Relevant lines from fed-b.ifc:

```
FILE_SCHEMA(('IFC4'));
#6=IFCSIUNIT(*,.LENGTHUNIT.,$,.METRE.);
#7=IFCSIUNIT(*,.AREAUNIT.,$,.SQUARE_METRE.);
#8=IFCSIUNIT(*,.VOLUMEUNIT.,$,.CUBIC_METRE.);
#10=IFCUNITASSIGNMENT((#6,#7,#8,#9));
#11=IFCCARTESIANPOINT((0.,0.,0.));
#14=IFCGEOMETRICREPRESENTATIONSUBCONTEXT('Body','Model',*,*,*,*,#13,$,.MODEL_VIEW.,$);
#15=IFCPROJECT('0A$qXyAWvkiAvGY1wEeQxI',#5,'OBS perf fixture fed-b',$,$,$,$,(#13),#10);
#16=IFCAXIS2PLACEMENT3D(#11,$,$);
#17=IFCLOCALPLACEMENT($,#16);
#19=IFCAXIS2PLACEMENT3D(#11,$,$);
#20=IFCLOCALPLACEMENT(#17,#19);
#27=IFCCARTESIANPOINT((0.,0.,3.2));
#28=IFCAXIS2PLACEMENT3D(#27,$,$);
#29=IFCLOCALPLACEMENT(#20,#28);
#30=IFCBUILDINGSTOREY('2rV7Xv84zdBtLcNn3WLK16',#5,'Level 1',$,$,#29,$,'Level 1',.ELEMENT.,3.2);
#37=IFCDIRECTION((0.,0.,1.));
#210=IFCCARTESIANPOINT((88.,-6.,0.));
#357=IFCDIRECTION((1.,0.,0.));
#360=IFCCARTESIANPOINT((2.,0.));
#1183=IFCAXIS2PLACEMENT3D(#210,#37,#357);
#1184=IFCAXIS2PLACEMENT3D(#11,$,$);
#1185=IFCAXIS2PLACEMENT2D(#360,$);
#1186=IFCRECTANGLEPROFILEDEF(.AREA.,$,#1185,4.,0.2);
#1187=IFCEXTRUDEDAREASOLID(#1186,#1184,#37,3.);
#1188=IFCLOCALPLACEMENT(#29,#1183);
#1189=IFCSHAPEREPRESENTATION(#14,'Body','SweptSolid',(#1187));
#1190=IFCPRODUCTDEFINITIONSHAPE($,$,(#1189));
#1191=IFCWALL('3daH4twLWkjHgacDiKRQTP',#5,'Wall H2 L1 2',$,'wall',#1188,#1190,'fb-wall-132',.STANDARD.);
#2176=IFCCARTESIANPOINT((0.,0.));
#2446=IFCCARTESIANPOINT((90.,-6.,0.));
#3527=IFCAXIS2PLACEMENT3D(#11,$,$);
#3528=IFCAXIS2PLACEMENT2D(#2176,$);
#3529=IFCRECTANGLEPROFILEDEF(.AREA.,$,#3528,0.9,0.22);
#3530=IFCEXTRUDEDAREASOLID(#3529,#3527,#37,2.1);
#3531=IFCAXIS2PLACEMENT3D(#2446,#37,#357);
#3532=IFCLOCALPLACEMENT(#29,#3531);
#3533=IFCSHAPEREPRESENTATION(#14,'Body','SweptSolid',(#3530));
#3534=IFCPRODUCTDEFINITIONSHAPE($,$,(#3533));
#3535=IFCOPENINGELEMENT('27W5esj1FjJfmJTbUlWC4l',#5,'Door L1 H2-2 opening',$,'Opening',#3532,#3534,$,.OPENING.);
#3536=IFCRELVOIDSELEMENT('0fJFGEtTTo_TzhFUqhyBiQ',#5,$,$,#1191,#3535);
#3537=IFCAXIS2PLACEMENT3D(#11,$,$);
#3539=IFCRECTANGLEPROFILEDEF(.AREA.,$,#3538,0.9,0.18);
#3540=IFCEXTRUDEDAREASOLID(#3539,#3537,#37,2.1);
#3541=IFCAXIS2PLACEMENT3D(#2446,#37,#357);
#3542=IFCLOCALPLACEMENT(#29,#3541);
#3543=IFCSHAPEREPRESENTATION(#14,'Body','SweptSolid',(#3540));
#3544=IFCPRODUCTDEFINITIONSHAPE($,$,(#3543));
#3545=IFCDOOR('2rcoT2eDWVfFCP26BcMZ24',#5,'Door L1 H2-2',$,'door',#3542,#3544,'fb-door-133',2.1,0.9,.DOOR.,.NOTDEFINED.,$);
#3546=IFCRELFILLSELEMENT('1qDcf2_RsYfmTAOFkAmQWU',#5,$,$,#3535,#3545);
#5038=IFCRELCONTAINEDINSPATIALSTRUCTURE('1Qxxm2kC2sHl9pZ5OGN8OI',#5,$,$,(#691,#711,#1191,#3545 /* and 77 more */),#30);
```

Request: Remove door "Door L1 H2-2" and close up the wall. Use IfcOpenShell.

```python
import ifcopenshell
import ifcopenshell.api.feature
import ifcopenshell.api.root
import ifcopenshell.geom
import ifcopenshell.util.shape

model = ifcopenshell.open("fed-b.ifc")
settings = ifcopenshell.geom.settings()


def volume(element):
    """Net volume in cubic metres, openings subtracted."""
    shape = ifcopenshell.geom.create_shape(settings, element)
    return ifcopenshell.util.shape.get_volume(shape.geometry)


door = model.by_guid("2rcoT2eDWVfFCP26BcMZ24")
opening = door.FillsVoids[0].RelatingOpeningElement
wall = opening.VoidsElements[0].RelatingBuildingElement
before = volume(wall)

ifcopenshell.api.root.remove_product(model, product=door)
ifcopenshell.api.feature.remove_feature(model, feature=opening)

after = volume(wall)

print(f"wall volume {before:.3f} -> {after:.3f} m3")

model.write("fed-b_rev.ifc")
```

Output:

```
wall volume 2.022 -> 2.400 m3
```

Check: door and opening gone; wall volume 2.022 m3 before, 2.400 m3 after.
